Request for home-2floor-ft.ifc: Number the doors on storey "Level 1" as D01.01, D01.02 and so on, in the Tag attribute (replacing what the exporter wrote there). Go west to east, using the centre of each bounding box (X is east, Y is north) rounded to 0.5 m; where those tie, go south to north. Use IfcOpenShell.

First a look at what the model holds.

```python
import ifcopenshell
import ifcopenshell.util.element
import ifcopenshell.util.placement

model = ifcopenshell.open("home-2floor-ft.ifc")
print(model.schema)
storey = next(s for s in model.by_type("IfcBuildingStorey") if s.Name == "Level 1")
doors = [e for e in ifcopenshell.util.element.get_decomposition(storey) if e.is_a("IfcDoor")]
for e in sorted(doors, key=lambda e: e.id()):
    origin = ifcopenshell.util.placement.get_local_placement(e.ObjectPlacement)[:3, 3]
    print(e.id(), e.Tag, e.Name, origin.round(2) + 0.0, sep=" | ")
```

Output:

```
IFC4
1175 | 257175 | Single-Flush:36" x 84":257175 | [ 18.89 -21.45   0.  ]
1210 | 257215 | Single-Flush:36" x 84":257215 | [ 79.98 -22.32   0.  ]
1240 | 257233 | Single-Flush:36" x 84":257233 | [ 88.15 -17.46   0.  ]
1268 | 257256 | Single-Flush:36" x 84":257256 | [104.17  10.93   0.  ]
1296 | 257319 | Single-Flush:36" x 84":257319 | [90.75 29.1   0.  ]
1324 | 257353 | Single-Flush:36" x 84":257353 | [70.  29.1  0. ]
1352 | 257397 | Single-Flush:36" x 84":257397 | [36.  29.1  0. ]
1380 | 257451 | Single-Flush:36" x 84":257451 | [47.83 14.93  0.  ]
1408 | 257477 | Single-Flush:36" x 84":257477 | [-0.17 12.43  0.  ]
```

```python
import ifcopenshell
import ifcopenshell.geom
import ifcopenshell.util.element
import ifcopenshell.util.shape

model = ifcopenshell.open("home-2floor-ft.ifc")
settings = ifcopenshell.geom.settings()
settings.set("use-world-coords", True)


def centre(element):
    shape = ifcopenshell.geom.create_shape(settings, element)
    return ifcopenshell.util.shape.get_bbox_centroid(shape.geometry)


storey = next(s for s in model.by_type("IfcBuildingStorey") if s.Name == "Level 1")
doors = [e for e in ifcopenshell.util.element.get_decomposition(storey) if e.is_a("IfcDoor")]

# Insertion points can sit at a corner or the storey origin, so sort by the geometry (in metres).
centres = {e: centre(e) for e in doors}
doors.sort(key=lambda e: (round(centres[e][0] / 0.5), centres[e][1]))

for i, e in enumerate(doors, start=1):
    number = f"D01.{i:02d}"
    e.Tag = number
    print(e.id(), number)

model.write("home-2floor-ft_updated.ifc")
```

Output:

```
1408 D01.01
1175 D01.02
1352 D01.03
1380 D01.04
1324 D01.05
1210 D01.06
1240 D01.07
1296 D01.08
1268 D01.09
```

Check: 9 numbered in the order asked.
